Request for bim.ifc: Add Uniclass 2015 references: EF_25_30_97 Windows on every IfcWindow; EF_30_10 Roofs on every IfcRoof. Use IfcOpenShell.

First a look at what the model holds.

```python
import ifcopenshell

model = ifcopenshell.open("bim.ifc")
print(model.schema)
print("classifications:", [c.Name for c in model.by_type("IfcClassification")])
for ifc_class in ("IfcDoor", "IfcRoof", "IfcStair", "IfcWall", "IfcWindow"):
    print(ifc_class, len(model.by_type(ifc_class)))
```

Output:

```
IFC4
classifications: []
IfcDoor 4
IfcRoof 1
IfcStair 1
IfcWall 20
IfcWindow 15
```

```python
import ifcopenshell
import ifcopenshell.api.classification

model = ifcopenshell.open("bim.ifc")

system = ifcopenshell.api.classification.add_classification(model, classification="Uniclass 2015")

codes = {
    "IfcWindow": ("EF_25_30_97", "Windows"),
    "IfcRoof": ("EF_30_10", "Roofs"),
}
for ifc_class, (code, name) in codes.items():
    products = model.by_type(ifc_class)
    ifcopenshell.api.classification.add_reference(
        model, products=products, classification=system, identification=code, name=name
    )
    print(code, len(products))

model.write("bim_updated.ifc")
```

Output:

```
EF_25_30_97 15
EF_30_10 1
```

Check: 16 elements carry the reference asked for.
